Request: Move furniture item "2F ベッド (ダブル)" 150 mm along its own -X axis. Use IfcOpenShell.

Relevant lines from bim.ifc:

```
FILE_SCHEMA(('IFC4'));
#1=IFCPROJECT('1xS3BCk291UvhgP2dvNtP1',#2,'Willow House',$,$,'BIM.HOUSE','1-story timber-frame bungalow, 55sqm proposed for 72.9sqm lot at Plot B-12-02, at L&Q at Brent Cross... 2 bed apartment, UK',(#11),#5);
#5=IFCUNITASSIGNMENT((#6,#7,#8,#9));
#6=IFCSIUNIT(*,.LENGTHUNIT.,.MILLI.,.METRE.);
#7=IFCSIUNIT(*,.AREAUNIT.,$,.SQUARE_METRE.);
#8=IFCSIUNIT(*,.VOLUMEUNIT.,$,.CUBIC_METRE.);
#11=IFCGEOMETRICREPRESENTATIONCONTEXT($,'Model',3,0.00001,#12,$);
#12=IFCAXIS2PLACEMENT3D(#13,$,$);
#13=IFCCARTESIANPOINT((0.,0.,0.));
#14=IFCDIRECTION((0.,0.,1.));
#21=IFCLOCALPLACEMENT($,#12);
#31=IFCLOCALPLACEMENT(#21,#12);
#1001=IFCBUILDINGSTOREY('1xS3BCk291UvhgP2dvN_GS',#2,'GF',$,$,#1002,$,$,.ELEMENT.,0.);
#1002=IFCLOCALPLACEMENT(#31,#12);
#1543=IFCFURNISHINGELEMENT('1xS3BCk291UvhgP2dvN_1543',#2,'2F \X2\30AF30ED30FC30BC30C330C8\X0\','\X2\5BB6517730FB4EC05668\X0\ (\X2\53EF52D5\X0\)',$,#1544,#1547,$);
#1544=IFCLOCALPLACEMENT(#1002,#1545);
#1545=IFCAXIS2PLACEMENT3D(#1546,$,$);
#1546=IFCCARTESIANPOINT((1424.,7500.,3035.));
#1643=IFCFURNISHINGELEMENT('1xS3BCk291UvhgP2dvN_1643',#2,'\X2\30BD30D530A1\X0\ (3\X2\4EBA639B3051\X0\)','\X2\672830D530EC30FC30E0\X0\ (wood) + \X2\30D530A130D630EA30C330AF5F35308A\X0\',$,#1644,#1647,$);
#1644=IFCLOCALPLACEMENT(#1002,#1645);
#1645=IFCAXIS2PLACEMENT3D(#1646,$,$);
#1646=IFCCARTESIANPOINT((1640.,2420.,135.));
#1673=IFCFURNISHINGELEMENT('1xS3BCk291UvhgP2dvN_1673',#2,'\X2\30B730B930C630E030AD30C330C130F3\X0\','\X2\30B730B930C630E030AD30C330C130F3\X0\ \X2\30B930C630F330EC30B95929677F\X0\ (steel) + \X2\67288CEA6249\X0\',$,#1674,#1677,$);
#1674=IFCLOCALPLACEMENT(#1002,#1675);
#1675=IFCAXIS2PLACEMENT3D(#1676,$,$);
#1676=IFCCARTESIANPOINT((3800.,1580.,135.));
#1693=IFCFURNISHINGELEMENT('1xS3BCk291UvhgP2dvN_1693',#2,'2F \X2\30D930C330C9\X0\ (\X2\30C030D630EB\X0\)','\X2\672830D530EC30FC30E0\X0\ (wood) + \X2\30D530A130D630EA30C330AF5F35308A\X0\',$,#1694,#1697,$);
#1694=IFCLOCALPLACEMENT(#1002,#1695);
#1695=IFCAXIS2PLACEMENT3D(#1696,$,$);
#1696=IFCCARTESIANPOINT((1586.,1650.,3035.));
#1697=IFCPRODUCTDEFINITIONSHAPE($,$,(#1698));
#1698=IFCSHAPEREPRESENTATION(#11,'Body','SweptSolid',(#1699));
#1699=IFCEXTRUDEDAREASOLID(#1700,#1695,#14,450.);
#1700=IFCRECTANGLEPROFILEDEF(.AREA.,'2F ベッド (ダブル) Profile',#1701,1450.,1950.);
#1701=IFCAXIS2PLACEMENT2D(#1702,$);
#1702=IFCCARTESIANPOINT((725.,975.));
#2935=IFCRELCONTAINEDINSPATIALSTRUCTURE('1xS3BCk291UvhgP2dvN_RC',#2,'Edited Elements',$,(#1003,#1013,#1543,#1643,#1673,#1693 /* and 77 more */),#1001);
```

```python
import ifcopenshell
import ifcopenshell.api.geometry
import ifcopenshell.util.placement
import ifcopenshell.util.unit

model = ifcopenshell.open("bim.ifc")
unit_scale = ifcopenshell.util.unit.calculate_unit_scale(model)

item = model.by_guid("1xS3BCk291UvhgP2dvN_1693")
matrix = ifcopenshell.util.placement.get_local_placement(item.ObjectPlacement)
matrix[:3, 3] -= matrix[:3, 0] * 0.15 / unit_scale
ifcopenshell.api.geometry.edit_object_placement(model, product=item, matrix=matrix, is_si=False)

print(ifcopenshell.util.placement.get_local_placement(item.ObjectPlacement).round(3) + 0.0)

model.write("bim_updated.ifc")
```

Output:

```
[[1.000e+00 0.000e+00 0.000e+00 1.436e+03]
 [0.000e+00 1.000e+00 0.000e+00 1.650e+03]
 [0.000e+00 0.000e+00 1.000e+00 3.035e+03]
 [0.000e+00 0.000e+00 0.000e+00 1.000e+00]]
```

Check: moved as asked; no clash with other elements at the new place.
